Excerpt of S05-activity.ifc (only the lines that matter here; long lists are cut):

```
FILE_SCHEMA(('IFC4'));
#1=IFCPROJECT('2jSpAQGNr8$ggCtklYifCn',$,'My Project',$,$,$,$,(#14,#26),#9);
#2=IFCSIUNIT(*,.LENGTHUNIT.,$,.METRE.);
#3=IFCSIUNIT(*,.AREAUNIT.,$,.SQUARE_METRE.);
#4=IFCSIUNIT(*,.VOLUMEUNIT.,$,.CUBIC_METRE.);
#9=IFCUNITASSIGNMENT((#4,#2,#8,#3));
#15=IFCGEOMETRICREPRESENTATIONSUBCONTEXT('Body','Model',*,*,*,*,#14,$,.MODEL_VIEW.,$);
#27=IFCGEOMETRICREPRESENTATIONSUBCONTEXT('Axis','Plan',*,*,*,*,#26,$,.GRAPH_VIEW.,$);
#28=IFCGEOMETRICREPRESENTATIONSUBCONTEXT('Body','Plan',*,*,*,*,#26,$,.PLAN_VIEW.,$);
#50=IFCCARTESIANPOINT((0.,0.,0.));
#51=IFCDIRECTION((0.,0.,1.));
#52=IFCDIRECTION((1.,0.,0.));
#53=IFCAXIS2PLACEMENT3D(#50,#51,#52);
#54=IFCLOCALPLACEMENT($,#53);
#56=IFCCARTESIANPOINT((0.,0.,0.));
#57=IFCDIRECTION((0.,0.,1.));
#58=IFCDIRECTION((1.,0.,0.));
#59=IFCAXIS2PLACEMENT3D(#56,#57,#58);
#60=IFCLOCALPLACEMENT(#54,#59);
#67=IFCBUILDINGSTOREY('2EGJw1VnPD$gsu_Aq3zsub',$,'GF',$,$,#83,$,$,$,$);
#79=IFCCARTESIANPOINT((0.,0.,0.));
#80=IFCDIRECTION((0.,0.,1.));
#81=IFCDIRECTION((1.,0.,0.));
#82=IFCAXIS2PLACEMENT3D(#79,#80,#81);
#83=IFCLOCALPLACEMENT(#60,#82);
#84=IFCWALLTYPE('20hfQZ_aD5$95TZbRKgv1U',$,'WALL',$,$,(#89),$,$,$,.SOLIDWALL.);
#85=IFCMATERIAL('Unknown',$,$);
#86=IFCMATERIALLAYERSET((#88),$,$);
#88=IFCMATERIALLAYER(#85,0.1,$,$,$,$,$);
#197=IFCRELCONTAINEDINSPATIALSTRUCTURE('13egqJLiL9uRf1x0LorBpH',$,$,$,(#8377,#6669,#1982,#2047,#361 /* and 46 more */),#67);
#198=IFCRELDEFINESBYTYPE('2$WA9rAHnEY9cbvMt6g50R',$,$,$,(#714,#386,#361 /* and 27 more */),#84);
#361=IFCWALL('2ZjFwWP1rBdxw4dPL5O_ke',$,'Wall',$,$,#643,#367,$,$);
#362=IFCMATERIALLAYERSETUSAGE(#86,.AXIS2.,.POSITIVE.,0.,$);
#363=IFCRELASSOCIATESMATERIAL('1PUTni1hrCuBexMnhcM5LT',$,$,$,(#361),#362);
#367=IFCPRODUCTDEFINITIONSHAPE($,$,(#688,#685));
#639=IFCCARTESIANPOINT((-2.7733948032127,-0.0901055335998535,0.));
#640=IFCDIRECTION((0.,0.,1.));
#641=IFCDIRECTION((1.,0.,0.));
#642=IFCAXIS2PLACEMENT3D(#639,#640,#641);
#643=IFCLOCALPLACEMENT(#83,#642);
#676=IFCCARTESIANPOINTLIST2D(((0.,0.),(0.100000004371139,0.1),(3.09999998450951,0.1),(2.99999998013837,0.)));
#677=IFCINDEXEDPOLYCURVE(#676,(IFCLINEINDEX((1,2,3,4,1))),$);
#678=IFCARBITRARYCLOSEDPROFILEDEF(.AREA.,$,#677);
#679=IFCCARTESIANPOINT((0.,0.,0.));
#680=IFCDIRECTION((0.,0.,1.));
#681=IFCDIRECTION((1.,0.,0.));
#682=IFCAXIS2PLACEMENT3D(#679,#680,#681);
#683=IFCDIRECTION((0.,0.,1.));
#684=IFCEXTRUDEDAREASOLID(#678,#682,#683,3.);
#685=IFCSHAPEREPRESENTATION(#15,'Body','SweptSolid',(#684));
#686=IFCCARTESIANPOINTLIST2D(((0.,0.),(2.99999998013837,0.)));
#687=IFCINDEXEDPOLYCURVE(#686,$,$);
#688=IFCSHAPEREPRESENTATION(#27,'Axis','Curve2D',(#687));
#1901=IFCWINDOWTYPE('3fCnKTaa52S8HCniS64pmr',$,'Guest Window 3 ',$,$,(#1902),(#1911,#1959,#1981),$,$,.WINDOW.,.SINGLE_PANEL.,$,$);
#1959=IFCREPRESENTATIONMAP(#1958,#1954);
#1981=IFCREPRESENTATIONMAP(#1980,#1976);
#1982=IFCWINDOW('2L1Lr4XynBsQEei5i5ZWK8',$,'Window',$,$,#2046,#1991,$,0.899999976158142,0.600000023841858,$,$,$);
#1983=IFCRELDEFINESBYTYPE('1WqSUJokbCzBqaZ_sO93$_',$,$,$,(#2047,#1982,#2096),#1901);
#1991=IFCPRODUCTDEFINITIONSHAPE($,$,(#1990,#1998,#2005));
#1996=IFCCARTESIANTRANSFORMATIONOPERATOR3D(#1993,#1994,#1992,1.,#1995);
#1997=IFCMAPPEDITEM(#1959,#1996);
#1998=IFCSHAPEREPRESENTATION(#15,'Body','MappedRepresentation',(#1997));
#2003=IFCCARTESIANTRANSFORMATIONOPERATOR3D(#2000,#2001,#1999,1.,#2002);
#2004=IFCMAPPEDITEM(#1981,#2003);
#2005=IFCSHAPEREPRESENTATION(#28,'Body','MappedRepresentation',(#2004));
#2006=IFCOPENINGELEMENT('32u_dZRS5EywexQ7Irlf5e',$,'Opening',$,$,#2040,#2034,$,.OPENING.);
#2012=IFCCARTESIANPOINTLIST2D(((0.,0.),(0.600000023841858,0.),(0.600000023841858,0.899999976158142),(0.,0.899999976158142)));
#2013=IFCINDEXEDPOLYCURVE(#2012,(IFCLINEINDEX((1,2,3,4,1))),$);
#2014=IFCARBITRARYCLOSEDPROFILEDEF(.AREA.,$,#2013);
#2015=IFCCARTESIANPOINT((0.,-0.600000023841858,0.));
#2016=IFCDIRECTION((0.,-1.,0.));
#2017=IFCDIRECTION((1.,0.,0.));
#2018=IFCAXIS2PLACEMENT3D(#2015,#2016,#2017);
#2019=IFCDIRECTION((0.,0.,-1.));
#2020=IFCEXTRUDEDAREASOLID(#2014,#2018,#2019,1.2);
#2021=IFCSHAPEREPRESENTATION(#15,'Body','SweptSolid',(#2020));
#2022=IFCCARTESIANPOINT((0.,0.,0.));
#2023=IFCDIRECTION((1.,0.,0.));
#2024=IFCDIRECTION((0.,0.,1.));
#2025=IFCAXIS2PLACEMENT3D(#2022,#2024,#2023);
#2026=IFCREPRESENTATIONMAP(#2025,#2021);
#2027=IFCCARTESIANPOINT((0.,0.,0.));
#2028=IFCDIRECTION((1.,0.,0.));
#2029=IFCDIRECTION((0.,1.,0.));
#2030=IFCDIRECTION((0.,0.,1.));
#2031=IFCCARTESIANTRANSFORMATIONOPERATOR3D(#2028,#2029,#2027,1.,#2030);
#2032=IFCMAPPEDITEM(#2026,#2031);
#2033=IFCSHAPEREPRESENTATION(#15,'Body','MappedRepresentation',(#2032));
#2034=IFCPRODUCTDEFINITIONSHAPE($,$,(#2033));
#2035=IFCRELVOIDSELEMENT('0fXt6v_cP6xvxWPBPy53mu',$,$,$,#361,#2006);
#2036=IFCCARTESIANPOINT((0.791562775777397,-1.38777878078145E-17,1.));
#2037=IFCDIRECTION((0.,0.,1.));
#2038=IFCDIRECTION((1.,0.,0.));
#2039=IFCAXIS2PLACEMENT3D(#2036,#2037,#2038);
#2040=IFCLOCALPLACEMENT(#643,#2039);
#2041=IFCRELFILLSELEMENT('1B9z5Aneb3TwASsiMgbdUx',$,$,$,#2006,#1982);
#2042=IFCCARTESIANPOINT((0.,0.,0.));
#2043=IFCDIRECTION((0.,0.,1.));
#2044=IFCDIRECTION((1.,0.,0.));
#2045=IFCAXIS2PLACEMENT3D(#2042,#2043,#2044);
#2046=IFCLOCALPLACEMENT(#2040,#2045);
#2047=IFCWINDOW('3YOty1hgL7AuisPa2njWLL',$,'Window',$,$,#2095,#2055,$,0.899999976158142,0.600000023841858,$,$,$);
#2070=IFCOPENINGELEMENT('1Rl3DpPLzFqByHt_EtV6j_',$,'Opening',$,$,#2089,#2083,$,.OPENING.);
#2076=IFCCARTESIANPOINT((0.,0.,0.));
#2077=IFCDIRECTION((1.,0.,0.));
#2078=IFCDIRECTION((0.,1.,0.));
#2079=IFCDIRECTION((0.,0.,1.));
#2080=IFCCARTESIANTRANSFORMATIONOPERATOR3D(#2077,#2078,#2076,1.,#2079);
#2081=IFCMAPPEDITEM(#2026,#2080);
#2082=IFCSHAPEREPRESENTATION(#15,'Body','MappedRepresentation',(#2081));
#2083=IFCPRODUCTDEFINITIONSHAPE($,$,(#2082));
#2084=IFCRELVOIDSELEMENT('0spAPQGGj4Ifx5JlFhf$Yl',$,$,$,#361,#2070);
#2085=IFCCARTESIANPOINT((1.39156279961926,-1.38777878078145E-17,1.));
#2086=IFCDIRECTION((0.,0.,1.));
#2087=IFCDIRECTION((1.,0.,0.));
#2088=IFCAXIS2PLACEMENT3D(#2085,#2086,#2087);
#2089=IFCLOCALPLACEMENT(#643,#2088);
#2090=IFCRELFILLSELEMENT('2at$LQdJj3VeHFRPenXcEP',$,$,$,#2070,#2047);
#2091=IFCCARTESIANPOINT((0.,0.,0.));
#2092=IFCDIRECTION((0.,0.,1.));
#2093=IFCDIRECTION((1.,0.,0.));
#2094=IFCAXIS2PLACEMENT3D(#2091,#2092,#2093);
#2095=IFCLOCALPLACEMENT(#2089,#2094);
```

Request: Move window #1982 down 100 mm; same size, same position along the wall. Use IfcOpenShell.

```python
import numpy as np
import ifcopenshell
import ifcopenshell.api.geometry
import ifcopenshell.util.placement
import ifcopenshell.util.unit

model = ifcopenshell.open("S05-activity.ifc")
unit_scale = ifcopenshell.util.unit.calculate_unit_scale(model)

window = model.by_id(1982)
opening = window.FillsVoids[0].RelatingOpeningElement
dz = -0.1

shift = np.array([0.0, 0.0, dz])
# The window is placed relative to its opening, so it follows when the opening moves.
matrix = ifcopenshell.util.placement.get_local_placement(opening.ObjectPlacement)
matrix[:3, 3] += shift
ifcopenshell.api.geometry.edit_object_placement(
    model, product=opening, matrix=matrix, is_si=False, should_transform_children=True
)

print(f"moved by {dz * unit_scale:+.3f} m")

model.write("S05-activity_rev.ifc")
```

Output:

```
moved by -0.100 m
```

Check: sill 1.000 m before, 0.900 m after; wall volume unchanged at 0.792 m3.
